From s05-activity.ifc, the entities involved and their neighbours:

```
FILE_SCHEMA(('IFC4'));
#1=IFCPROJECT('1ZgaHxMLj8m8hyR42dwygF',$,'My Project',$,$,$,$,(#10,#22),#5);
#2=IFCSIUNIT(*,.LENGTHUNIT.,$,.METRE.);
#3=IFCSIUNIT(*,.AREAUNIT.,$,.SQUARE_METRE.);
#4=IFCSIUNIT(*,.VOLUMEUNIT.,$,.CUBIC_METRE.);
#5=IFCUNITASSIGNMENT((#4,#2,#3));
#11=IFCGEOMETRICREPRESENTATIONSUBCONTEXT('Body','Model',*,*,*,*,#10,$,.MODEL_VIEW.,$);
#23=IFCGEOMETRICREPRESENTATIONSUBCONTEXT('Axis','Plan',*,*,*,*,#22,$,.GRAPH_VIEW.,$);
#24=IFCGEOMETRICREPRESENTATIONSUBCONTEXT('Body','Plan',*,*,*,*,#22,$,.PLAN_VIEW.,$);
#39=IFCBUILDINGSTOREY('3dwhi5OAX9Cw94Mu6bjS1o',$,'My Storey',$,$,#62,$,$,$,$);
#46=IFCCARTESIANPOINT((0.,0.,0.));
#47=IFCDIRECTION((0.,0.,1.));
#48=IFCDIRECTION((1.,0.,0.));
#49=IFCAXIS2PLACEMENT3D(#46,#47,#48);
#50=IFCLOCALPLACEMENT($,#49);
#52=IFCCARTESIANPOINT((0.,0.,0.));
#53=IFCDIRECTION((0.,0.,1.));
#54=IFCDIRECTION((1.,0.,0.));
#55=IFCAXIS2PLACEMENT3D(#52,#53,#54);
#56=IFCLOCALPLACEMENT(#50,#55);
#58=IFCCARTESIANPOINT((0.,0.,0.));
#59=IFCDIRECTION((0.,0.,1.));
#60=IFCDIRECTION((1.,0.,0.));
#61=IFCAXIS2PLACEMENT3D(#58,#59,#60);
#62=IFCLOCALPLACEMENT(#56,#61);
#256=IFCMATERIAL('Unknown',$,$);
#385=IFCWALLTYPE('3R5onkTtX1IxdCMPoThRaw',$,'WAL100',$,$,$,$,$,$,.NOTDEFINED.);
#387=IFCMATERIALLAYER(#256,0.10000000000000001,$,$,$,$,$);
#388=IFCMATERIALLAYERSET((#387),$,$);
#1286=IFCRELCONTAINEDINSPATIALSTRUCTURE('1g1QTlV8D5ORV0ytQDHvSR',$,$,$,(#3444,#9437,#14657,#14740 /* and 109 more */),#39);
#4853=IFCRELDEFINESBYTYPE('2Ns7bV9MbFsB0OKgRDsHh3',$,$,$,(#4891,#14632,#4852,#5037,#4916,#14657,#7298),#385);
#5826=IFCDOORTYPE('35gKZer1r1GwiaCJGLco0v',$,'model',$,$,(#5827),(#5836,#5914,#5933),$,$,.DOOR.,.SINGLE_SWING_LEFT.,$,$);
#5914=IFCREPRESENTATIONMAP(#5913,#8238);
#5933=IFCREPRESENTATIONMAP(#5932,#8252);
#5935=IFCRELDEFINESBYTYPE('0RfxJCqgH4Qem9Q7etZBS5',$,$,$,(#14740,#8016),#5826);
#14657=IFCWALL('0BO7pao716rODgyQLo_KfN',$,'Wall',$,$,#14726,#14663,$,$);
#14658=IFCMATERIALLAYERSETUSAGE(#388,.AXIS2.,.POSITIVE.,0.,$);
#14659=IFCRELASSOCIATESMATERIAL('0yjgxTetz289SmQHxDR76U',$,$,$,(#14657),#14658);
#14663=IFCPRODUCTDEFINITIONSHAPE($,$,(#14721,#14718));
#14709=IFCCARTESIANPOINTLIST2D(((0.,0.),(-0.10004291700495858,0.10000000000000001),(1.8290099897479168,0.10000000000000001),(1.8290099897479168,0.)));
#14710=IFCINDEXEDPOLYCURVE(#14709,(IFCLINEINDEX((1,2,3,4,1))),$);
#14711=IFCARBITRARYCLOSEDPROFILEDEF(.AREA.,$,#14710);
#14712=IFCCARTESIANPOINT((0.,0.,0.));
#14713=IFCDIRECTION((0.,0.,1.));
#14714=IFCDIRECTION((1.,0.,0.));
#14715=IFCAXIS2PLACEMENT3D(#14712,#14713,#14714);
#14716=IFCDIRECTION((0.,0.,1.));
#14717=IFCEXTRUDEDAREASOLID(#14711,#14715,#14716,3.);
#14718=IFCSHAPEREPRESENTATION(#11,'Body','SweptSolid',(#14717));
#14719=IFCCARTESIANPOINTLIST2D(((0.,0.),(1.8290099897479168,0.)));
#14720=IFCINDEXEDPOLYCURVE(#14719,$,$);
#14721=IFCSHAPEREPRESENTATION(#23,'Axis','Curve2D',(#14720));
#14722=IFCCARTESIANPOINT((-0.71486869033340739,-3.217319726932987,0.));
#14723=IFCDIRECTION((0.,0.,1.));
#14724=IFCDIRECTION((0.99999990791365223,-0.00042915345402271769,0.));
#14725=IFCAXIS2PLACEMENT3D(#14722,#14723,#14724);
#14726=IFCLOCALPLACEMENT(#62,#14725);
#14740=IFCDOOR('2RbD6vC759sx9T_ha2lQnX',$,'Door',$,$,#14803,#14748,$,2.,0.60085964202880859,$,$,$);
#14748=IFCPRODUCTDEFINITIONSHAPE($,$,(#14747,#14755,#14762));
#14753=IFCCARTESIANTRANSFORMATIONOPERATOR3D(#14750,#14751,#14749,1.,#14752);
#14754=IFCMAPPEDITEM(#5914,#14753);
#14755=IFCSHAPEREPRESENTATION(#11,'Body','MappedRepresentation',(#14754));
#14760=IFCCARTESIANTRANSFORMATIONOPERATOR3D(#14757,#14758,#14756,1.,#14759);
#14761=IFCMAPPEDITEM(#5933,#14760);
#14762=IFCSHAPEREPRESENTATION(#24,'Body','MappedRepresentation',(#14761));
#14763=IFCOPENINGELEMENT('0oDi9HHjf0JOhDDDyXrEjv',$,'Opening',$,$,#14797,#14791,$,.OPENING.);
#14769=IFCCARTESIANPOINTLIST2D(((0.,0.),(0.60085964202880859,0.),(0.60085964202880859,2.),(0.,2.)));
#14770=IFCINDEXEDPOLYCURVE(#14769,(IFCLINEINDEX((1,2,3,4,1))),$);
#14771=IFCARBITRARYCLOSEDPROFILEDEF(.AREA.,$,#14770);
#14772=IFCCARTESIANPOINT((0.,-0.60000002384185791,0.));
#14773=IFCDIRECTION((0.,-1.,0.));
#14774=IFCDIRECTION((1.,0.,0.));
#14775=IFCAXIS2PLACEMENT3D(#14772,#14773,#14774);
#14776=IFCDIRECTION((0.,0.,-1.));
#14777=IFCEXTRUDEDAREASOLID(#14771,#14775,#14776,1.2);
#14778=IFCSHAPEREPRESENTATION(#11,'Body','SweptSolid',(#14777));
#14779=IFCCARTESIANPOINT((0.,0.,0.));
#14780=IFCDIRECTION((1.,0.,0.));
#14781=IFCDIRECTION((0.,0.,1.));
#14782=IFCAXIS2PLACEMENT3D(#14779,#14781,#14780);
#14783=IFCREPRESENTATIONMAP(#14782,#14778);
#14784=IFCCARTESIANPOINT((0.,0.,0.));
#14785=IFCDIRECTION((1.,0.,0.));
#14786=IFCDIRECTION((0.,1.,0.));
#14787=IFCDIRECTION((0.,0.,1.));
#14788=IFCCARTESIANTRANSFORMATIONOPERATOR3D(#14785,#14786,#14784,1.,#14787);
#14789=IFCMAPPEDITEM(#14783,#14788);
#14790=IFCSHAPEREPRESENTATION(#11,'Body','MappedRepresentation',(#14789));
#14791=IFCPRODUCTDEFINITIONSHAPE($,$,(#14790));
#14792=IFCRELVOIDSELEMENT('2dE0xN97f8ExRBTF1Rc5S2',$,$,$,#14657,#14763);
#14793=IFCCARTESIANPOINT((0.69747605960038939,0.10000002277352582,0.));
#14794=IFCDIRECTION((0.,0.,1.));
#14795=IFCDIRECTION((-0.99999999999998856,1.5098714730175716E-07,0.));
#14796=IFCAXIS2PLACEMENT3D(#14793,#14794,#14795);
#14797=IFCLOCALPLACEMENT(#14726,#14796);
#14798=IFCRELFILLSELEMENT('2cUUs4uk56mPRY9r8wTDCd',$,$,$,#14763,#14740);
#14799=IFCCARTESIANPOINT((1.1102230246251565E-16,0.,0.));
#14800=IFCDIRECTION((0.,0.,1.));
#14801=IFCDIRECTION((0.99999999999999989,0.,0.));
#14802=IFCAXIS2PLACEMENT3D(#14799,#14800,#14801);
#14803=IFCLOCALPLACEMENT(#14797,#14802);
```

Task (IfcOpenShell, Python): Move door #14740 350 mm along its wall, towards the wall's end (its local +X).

```python
import ifcopenshell
import ifcopenshell.api.geometry
import ifcopenshell.util.placement
import ifcopenshell.util.unit

model = ifcopenshell.open("s05-activity.ifc")
unit_scale = ifcopenshell.util.unit.calculate_unit_scale(model)

door = model.by_guid("2RbD6vC759sx9T_ha2lQnX")
opening = door.FillsVoids[0].RelatingOpeningElement
wall = opening.VoidsElements[0].RelatingBuildingElement

wall_matrix = ifcopenshell.util.placement.get_local_placement(wall.ObjectPlacement)
shift = wall_matrix[:3, 0] * 0.35 / unit_scale
before = ifcopenshell.util.placement.get_local_placement(door.ObjectPlacement)[:3, 3].copy()

# The door is placed relative to its opening, so it follows when the opening moves.
matrix = ifcopenshell.util.placement.get_local_placement(opening.ObjectPlacement)
matrix[:3, 3] += shift
ifcopenshell.api.geometry.edit_object_placement(
    model, product=opening, matrix=matrix, is_si=False, should_transform_children=True
)

after = ifcopenshell.util.placement.get_local_placement(door.ObjectPlacement)[:3, 3]
print("door moved by", (after - before).round(3) + 0.0)

model.write("s05-activity_updated.ifc")
```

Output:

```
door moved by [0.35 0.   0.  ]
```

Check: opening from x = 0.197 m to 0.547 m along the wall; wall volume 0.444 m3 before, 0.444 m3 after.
